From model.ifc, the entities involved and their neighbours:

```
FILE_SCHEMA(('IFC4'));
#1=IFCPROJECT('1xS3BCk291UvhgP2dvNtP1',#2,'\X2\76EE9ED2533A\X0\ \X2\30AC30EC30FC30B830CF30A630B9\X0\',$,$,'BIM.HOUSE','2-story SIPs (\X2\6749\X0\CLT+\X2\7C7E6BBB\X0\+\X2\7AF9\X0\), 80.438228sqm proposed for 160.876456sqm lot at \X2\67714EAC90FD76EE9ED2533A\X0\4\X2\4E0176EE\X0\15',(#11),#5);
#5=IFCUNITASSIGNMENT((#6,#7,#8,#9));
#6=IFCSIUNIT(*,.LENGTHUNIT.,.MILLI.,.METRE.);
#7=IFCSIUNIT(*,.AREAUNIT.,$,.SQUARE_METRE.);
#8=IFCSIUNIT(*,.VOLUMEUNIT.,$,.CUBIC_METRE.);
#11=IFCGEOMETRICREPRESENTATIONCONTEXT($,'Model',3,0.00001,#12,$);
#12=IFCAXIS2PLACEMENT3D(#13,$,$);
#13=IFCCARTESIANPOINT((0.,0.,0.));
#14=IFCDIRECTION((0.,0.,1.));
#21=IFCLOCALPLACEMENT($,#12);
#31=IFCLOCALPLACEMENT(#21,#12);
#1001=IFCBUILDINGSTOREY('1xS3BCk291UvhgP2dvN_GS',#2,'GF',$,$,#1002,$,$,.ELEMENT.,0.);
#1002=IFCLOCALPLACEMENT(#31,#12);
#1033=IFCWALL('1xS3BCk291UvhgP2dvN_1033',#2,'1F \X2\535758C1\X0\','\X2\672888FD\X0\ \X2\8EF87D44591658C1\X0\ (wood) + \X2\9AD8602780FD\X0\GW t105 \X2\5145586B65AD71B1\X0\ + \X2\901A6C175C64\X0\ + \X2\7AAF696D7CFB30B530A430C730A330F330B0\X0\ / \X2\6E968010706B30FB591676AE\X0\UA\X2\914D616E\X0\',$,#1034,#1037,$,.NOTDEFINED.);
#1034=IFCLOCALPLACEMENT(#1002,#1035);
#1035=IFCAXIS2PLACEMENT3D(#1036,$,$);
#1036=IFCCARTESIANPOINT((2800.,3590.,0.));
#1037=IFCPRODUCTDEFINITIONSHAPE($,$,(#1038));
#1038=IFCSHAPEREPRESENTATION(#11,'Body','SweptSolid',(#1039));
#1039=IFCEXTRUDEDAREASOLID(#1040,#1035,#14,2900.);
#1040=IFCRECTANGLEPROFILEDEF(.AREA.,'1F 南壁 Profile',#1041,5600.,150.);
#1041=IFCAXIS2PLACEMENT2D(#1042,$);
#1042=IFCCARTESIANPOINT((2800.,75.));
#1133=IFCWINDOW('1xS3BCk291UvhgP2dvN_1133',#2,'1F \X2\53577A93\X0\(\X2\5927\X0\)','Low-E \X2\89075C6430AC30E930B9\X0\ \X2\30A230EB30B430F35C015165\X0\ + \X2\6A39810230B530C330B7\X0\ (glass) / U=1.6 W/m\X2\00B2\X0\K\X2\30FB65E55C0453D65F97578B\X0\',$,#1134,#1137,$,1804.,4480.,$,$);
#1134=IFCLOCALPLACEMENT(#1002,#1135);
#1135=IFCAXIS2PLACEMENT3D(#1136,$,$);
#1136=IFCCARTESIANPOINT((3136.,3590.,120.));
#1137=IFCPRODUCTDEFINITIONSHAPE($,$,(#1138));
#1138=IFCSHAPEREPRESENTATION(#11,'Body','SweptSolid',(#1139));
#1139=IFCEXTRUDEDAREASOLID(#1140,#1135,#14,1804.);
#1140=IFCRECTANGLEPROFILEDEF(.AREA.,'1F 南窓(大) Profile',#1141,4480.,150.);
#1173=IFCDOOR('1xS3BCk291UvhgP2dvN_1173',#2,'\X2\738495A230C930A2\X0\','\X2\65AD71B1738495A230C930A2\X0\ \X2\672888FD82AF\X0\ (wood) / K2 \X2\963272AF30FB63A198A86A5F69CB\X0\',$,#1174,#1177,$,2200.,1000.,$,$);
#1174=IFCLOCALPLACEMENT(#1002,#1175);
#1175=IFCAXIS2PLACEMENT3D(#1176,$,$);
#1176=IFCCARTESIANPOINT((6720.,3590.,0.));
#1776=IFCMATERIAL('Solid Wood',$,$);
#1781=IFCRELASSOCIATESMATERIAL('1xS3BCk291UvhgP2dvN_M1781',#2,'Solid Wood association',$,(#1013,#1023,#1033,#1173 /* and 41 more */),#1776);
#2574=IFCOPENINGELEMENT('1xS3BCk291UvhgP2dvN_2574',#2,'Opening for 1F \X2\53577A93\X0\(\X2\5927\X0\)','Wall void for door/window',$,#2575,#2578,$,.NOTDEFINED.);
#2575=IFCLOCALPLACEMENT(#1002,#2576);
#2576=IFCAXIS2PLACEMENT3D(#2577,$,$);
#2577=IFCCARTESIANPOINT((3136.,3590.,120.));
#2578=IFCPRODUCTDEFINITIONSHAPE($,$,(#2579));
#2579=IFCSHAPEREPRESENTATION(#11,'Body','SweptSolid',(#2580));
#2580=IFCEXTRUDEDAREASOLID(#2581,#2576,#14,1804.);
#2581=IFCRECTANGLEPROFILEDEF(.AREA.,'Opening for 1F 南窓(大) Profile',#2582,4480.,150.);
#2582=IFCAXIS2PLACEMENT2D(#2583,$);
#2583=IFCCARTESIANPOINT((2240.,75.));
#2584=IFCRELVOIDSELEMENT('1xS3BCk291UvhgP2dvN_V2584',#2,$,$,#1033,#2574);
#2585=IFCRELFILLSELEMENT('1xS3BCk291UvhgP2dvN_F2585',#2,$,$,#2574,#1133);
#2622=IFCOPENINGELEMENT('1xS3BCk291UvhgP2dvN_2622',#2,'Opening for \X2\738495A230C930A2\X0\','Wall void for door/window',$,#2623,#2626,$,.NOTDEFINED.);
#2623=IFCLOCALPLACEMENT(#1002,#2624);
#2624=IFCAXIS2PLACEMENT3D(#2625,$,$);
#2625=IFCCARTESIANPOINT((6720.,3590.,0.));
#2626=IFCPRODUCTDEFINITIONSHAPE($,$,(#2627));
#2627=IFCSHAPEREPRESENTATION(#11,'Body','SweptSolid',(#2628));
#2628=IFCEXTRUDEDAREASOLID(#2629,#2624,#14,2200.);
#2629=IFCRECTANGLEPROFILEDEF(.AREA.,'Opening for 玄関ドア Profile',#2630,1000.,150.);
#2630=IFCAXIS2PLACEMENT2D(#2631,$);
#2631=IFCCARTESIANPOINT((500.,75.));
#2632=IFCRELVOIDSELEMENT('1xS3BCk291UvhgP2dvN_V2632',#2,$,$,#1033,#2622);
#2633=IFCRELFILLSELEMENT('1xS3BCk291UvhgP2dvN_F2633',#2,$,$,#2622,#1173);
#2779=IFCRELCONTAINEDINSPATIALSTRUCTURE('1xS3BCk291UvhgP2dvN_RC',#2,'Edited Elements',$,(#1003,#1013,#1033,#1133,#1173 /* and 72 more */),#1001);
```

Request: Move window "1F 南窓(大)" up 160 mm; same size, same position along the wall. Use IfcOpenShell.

```python
import numpy as np
import ifcopenshell
import ifcopenshell.api.geometry
import ifcopenshell.util.placement
import ifcopenshell.util.unit

model = ifcopenshell.open("model.ifc")
unit_scale = ifcopenshell.util.unit.calculate_unit_scale(model)

window = model.by_guid("1xS3BCk291UvhgP2dvN_1133")
opening = window.FillsVoids[0].RelatingOpeningElement
dz = 160.0

shift = np.array([0.0, 0.0, dz])
# The window is not placed relative to its opening, so move both.
for product in (opening, window):
    matrix = ifcopenshell.util.placement.get_local_placement(product.ObjectPlacement)
    matrix[:3, 3] += shift
    ifcopenshell.api.geometry.edit_object_placement(model, product=product, matrix=matrix, is_si=False)

print(f"moved by {dz * unit_scale:+.3f} m")

model.write("model_rev.ifc")
```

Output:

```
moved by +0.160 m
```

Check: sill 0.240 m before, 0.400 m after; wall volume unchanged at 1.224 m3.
